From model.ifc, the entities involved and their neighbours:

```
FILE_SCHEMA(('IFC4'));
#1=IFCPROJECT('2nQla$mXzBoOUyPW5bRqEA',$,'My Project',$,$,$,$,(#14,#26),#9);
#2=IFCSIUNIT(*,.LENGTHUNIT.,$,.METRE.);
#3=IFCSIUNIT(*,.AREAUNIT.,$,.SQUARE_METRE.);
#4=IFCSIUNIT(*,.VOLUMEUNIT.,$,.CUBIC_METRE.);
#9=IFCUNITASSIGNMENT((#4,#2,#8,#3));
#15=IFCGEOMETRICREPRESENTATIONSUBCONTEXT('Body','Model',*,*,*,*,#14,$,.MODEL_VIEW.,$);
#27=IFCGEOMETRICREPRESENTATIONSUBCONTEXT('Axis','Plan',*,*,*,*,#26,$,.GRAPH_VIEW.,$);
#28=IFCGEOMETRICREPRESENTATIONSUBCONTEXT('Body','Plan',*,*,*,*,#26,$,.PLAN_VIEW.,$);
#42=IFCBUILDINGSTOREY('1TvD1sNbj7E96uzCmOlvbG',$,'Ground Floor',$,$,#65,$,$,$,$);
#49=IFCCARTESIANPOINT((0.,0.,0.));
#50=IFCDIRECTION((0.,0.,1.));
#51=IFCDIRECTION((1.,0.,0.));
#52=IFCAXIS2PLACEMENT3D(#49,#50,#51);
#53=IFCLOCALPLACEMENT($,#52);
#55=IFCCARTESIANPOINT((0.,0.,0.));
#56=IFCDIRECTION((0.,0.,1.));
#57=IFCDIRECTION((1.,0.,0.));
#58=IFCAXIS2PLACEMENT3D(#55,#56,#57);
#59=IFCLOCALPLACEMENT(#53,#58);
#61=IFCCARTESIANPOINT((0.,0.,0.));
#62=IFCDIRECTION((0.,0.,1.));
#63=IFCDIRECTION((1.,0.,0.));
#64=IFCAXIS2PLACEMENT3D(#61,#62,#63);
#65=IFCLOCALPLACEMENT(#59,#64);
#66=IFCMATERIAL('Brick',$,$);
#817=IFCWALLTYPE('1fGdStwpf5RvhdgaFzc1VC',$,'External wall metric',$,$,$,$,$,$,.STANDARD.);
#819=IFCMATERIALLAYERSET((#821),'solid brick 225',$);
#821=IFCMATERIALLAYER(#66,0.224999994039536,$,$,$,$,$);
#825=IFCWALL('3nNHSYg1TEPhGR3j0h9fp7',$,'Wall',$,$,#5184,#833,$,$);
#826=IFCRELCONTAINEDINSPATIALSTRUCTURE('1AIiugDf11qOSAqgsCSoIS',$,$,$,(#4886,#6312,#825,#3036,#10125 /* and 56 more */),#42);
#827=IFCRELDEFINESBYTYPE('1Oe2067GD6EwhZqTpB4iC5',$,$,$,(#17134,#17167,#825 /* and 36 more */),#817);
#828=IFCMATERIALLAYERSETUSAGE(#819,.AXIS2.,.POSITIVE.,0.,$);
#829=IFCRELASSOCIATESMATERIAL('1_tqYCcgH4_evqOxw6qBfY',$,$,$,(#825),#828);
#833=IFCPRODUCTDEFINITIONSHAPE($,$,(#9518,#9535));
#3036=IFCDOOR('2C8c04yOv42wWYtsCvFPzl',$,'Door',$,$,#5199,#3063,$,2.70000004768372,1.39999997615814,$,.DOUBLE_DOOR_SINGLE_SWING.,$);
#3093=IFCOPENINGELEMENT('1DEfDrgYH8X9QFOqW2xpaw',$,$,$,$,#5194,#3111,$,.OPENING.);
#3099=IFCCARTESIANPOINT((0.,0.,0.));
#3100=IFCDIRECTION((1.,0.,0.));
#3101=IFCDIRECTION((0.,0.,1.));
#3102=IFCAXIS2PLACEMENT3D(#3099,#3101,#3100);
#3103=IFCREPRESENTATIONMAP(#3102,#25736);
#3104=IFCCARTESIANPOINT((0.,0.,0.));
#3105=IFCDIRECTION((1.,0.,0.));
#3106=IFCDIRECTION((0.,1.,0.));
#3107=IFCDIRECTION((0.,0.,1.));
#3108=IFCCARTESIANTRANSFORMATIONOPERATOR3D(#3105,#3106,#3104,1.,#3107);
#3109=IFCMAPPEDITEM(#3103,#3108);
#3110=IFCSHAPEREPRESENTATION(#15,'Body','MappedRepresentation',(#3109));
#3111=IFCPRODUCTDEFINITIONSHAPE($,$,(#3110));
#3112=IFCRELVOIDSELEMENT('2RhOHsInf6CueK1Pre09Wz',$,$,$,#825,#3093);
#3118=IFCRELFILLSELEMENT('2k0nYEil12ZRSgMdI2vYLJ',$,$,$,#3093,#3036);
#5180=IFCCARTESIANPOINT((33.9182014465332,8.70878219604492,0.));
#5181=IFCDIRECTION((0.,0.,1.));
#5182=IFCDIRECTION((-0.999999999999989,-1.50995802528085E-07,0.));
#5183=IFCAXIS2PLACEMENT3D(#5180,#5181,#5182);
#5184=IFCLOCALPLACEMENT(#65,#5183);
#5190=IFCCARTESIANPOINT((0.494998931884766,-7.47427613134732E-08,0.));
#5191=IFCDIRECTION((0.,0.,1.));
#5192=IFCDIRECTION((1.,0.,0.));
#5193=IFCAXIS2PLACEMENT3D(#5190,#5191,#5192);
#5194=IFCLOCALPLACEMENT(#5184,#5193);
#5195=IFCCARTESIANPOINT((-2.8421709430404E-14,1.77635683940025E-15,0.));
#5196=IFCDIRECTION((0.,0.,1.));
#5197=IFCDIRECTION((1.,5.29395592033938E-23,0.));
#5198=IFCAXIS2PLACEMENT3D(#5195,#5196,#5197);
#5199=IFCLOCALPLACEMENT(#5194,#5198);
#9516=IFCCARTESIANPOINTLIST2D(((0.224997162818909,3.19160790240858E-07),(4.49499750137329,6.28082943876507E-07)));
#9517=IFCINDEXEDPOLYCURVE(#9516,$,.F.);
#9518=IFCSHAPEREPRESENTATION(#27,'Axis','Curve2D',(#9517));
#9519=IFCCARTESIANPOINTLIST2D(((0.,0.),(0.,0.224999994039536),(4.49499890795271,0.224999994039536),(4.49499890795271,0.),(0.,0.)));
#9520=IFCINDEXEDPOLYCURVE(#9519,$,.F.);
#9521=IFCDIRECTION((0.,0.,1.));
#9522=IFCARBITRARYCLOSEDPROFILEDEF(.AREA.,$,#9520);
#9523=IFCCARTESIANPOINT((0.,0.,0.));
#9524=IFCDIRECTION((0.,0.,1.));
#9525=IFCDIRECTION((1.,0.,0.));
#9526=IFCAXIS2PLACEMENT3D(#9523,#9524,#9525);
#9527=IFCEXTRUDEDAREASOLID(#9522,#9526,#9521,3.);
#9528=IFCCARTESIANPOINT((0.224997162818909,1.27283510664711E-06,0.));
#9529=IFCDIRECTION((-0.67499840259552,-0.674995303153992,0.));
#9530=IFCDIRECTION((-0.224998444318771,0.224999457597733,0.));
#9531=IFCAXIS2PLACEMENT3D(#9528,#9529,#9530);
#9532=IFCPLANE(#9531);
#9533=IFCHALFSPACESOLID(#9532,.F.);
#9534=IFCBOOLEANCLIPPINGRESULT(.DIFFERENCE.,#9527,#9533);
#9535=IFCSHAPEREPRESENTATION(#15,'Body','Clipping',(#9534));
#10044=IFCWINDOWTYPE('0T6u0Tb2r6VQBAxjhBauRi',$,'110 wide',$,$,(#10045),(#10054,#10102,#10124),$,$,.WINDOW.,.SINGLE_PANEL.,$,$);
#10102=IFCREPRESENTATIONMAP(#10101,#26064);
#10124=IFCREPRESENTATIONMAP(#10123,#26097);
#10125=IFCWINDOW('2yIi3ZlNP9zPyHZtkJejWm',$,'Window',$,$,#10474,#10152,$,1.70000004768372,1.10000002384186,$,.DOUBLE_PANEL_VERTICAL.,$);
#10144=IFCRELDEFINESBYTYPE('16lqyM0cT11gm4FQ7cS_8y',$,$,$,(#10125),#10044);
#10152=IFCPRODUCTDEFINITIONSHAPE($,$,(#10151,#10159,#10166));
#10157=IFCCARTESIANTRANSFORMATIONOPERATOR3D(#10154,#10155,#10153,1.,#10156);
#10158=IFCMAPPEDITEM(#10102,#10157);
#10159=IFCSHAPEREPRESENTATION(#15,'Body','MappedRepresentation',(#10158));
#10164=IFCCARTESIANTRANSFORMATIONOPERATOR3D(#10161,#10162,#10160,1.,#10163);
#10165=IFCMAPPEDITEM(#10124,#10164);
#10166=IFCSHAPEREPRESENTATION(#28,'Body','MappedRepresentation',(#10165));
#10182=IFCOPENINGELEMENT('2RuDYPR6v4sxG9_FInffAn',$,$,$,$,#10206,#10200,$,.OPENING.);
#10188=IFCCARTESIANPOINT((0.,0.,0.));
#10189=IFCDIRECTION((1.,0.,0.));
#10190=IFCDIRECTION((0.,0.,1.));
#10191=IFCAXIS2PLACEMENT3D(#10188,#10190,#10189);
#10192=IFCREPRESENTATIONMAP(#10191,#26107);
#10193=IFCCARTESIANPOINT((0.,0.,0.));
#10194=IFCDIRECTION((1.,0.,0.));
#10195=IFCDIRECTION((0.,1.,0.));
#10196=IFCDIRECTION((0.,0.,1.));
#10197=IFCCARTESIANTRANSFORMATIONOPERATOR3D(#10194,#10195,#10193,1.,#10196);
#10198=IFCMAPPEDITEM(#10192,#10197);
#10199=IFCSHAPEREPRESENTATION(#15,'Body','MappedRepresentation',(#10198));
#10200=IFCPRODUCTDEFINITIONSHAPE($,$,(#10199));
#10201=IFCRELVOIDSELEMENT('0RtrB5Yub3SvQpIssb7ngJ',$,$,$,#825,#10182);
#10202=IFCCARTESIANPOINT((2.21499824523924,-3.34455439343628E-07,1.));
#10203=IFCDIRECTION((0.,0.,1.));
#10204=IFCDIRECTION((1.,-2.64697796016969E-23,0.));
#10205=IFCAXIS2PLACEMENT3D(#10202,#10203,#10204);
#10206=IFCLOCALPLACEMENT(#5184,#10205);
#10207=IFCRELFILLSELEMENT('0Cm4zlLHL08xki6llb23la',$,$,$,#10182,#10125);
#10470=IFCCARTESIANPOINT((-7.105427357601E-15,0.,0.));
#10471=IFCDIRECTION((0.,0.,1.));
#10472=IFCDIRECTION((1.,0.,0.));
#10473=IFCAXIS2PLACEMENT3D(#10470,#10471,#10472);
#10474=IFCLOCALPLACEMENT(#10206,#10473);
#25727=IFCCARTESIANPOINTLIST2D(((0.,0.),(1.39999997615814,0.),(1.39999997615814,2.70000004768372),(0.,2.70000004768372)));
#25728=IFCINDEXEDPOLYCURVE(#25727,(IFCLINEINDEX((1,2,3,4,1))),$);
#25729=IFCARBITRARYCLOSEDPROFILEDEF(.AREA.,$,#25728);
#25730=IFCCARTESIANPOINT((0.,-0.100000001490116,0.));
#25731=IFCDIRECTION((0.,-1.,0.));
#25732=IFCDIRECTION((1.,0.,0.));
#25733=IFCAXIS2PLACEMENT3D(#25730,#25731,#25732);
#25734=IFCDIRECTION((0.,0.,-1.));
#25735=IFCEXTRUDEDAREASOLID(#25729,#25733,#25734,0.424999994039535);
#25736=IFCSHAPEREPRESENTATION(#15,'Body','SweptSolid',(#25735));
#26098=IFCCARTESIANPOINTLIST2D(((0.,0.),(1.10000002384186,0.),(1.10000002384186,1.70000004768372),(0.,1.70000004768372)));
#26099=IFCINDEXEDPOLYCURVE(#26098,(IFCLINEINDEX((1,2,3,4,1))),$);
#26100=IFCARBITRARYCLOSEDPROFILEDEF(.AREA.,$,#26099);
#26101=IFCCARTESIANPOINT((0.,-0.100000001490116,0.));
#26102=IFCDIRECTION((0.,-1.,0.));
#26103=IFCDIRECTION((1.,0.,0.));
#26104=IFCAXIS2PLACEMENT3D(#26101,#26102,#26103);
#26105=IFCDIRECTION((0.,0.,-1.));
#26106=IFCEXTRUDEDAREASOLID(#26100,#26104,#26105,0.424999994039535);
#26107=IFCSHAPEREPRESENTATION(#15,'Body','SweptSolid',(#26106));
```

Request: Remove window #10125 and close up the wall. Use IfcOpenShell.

```python
import ifcopenshell
import ifcopenshell.api.feature
import ifcopenshell.api.root
import ifcopenshell.geom
import ifcopenshell.util.shape

model = ifcopenshell.open("model.ifc")
settings = ifcopenshell.geom.settings()


def volume(element):
    """Net volume in cubic metres, openings subtracted."""
    shape = ifcopenshell.geom.create_shape(settings, element)
    return ifcopenshell.util.shape.get_volume(shape.geometry)


window = model.by_guid("2yIi3ZlNP9zPyHZtkJejWm")
opening = window.FillsVoids[0].RelatingOpeningElement
wall = opening.VoidsElements[0].RelatingBuildingElement
before = volume(wall)

ifcopenshell.api.root.remove_product(model, product=window)
ifcopenshell.api.feature.remove_feature(model, feature=opening)

after = volume(wall)

print(f"wall volume {before:.3f} -> {after:.3f} m3")

model.write("model_edited.ifc")
```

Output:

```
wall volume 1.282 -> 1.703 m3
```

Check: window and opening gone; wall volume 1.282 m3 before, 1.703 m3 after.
